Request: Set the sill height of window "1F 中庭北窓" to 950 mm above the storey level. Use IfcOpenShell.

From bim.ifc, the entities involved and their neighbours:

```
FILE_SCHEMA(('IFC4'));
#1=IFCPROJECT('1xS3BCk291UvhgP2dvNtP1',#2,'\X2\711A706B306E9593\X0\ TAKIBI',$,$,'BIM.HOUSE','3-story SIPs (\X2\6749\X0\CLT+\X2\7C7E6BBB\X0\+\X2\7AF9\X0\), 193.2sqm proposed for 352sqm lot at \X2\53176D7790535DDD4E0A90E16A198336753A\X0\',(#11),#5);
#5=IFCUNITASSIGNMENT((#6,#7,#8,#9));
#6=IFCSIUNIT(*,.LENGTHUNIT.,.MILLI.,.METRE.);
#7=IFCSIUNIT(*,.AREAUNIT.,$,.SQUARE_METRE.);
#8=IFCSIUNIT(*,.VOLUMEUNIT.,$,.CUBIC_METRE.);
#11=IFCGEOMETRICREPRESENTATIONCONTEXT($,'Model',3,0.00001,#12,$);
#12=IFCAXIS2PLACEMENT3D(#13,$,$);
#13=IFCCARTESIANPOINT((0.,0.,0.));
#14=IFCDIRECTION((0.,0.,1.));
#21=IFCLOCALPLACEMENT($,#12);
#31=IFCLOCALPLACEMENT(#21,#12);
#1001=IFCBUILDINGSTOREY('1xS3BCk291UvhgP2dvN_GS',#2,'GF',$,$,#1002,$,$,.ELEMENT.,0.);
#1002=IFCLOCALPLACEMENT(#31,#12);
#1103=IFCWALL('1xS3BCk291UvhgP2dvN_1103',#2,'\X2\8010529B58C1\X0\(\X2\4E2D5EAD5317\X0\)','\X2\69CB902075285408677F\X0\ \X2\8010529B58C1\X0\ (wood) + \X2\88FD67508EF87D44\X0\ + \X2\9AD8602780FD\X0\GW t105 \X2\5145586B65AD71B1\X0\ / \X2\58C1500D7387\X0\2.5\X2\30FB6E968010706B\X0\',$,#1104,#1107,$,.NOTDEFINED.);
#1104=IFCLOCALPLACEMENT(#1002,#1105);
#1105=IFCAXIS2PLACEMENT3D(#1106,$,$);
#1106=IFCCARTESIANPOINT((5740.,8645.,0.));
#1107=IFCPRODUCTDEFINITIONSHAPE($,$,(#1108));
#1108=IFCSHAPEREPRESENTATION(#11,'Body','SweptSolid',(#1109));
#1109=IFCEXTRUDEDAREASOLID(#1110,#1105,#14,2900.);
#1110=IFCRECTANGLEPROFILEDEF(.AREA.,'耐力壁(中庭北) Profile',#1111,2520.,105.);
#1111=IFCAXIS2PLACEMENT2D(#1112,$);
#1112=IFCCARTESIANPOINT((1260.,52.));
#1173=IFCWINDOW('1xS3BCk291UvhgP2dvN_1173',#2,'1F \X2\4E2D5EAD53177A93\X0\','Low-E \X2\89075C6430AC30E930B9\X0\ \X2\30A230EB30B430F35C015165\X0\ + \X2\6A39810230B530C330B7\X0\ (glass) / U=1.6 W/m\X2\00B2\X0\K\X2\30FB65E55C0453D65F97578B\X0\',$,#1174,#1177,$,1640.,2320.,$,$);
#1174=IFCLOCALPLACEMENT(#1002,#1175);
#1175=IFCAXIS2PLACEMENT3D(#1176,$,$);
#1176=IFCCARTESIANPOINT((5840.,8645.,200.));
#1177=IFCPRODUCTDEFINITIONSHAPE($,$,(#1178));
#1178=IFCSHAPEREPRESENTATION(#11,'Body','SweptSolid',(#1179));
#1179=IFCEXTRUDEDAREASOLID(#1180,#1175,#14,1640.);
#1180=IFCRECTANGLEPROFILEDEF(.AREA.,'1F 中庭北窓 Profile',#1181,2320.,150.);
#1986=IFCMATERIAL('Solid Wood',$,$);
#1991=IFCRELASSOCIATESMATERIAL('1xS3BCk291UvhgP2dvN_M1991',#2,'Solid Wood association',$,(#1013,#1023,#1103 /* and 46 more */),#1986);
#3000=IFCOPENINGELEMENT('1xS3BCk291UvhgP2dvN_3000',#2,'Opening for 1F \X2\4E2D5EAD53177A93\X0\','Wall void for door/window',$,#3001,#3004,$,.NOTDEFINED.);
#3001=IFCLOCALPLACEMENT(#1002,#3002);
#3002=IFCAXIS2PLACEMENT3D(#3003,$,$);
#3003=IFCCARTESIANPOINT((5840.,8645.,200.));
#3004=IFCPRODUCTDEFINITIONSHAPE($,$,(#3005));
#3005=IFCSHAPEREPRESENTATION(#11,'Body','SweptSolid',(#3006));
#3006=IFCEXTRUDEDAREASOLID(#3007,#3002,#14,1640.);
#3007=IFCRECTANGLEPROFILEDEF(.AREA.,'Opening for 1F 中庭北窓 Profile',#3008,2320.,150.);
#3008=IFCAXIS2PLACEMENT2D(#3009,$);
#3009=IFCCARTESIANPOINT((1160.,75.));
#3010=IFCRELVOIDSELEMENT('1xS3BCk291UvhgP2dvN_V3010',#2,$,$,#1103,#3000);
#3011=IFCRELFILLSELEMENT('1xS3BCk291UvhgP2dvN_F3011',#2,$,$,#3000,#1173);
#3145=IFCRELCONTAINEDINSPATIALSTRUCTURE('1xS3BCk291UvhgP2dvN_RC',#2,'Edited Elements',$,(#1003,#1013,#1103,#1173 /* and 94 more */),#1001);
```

```python
import numpy as np
import ifcopenshell
import ifcopenshell.api.geometry
import ifcopenshell.geom
import ifcopenshell.util.element
import ifcopenshell.util.placement
import ifcopenshell.util.shape
import ifcopenshell.util.unit

model = ifcopenshell.open("bim.ifc")
unit_scale = ifcopenshell.util.unit.calculate_unit_scale(model)

window = model.by_id(1173)
opening = window.FillsVoids[0].RelatingOpeningElement
storey = ifcopenshell.util.element.get_container(window, ifc_class="IfcBuildingStorey")
level = ifcopenshell.util.placement.get_local_placement(storey.ObjectPlacement)[2, 3]

# The opening's origin need not be at the sill, so measure its lowest point.
shape = ifcopenshell.geom.create_shape(ifcopenshell.geom.settings(), opening)
bottom = ifcopenshell.util.shape.get_shape_bottom_elevation(shape, shape.geometry) / unit_scale
dz = level + 0.95 / unit_scale - bottom

shift = np.array([0.0, 0.0, dz])
# The window is not placed relative to its opening, so move both.
for product in (opening, window):
    matrix = ifcopenshell.util.placement.get_local_placement(product.ObjectPlacement)
    matrix[:3, 3] += shift
    ifcopenshell.api.geometry.edit_object_placement(model, product=product, matrix=matrix, is_si=False)

print(f"moved by {dz * unit_scale:+.3f} m")

model.write("bim-out.ifc")
```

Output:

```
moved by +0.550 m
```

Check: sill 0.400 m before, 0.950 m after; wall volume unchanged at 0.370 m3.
